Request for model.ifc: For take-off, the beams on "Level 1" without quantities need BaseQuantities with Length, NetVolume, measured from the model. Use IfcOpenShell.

First a look at what the model holds.

```python
import ifcopenshell
import ifcopenshell.util.element
import ifcopenshell.util.unit

model = ifcopenshell.open("model.ifc")
print(model.schema)
for unit_type in ("LENGTHUNIT", "AREAUNIT", "VOLUMEUNIT"):
    print(unit_type, ifcopenshell.util.unit.calculate_unit_scale(model, unit_type))
storey = next(s for s in model.by_type("IfcBuildingStorey") if s.Name == "Level 1")
beams = [e for e in ifcopenshell.util.element.get_decomposition(storey) if e.is_a("IfcBeam")]
for e in sorted(beams, key=lambda e: e.id()):
    print(e.id(), e.is_a(), e.Name, list(ifcopenshell.util.element.get_psets(e, qtos_only=True)), sep=" | ")
```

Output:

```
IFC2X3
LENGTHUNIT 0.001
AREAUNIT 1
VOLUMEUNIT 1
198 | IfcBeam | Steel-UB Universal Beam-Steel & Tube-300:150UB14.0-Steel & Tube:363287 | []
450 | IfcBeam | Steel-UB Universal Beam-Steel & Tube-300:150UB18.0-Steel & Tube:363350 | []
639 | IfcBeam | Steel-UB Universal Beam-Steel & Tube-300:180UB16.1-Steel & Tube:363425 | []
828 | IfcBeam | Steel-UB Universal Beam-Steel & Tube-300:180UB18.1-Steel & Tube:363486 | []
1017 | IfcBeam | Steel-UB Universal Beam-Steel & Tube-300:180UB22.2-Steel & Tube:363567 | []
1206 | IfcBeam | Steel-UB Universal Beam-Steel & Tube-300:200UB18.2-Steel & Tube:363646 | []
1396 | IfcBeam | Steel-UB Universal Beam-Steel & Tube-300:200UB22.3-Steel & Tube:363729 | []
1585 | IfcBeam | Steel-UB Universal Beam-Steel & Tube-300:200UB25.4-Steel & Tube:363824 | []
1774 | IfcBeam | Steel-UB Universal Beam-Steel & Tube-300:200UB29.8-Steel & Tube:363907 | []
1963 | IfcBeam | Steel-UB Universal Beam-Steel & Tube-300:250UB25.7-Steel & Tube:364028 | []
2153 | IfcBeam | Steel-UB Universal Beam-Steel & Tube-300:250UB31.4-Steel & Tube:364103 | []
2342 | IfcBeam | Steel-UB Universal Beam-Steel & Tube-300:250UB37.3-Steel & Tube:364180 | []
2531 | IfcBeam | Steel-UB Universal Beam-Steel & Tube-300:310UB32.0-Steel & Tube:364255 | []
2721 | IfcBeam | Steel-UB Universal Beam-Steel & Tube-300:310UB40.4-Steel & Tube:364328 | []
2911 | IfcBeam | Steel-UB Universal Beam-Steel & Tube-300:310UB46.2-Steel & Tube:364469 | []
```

```python
import ifcopenshell
import ifcopenshell.api.pset
import ifcopenshell.geom
import ifcopenshell.util.element
import ifcopenshell.util.shape
import ifcopenshell.util.unit

model = ifcopenshell.open("model.ifc")
unit_scale = ifcopenshell.util.unit.calculate_unit_scale(model)
volume_scale = ifcopenshell.util.unit.calculate_unit_scale(model, "VOLUMEUNIT")
settings = ifcopenshell.geom.settings()

storey = next(s for s in model.by_type("IfcBuildingStorey") if s.Name == "Level 1")
beams = [e for e in ifcopenshell.util.element.get_decomposition(storey) if e.is_a("IfcBeam")]

for e in sorted(beams, key=lambda e: e.id()):
    if ifcopenshell.util.element.get_psets(e, qtos_only=True, should_inherit=False):
        continue
    # Geometry comes back in metres, in the element's own axes.
    shape = ifcopenshell.geom.create_shape(settings, e)
    values = {
        "Length": ifcopenshell.util.shape.get_max_xyz(shape.geometry) / unit_scale,
        "NetVolume": ifcopenshell.util.shape.get_volume(shape.geometry) / volume_scale,
    }
    qto = ifcopenshell.api.pset.add_qto(model, product=e, name="BaseQuantities")
    ifcopenshell.api.pset.edit_qto(model, qto=qto, properties=values)
    print(e.id(), {k: round(v, 3) for k, v in values.items()})

model.write("model_rev.ifc")
```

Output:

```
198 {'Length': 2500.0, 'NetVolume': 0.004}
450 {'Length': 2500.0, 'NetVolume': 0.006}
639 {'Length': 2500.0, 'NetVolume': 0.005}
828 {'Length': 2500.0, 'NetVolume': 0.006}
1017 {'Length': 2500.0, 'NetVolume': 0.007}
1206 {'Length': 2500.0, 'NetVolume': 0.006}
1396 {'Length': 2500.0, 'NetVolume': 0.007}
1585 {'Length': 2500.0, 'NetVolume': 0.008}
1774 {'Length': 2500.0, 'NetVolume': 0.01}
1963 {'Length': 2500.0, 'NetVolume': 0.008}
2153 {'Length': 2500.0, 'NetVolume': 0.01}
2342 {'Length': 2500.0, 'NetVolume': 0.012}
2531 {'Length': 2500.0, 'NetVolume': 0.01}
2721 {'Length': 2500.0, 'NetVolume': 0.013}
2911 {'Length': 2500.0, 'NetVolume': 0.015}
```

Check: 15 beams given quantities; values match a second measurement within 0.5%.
